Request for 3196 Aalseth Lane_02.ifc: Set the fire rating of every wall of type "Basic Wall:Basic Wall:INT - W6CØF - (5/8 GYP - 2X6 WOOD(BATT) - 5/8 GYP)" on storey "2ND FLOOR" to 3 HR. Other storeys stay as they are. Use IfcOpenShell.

First a look at what the model holds.

```python
import ifcopenshell
import ifcopenshell.util.element

model = ifcopenshell.open("3196 Aalseth Lane_02.ifc")
print(model.schema)
storey = next(s for s in model.by_type("IfcBuildingStorey") if s.Name == "2ND FLOOR")
walls = [e for e in ifcopenshell.util.element.get_decomposition(storey) if e.is_a("IfcWall")]
seen = {}
for e in walls:
    element_type = ifcopenshell.util.element.get_type(e)
    key = (element_type.Name if element_type != e and element_type else None, ifcopenshell.util.element.get_pset(e, "Pset_WallCommon", "FireRating"))
    seen[key] = seen.get(key, 0) + 1
for (name, value), count in sorted(seen.items(), key=str):
    print(count, "x", name, "|", value)
```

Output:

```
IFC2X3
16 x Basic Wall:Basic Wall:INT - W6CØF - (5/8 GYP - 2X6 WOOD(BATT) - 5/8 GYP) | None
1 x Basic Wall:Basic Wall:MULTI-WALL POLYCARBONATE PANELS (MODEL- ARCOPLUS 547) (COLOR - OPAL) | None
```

```python
import ifcopenshell
import ifcopenshell.api.pset
import ifcopenshell.util.element

model = ifcopenshell.open("3196 Aalseth Lane_02.ifc")

storey = next(s for s in model.by_type("IfcBuildingStorey") if s.Name == "2ND FLOOR")
walls = [e for e in ifcopenshell.util.element.get_decomposition(storey) if e.is_a("IfcWall")]

count = 0
for e in walls:
    element_type = ifcopenshell.util.element.get_type(e)
    if element_type in (None, e) or element_type.Name != "Basic Wall:Basic Wall:INT - W6CØF - (5/8 GYP - 2X6 WOOD(BATT) - 5/8 GYP)":
        continue
    # add_pset returns the element's existing set when there is one.
    pset = ifcopenshell.api.pset.add_pset(model, product=e, name="Pset_WallCommon")
    ifcopenshell.api.pset.edit_pset(model, pset=pset, properties={"FireRating": "3 HR"})
    count += 1

print(count, "walls updated")

model.write("3196 Aalseth Lane_02_rev.ifc")
```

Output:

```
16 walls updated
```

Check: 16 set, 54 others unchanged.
